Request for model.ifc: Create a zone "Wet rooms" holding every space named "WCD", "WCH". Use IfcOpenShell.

First a look at what the model holds.

```python
import ifcopenshell

model = ifcopenshell.open("model.ifc")
print(model.schema)
seen = {}
for space in model.by_type("IfcSpace"):
    seen[space.LongName] = seen.get(space.LongName, 0) + 1
for name, count in sorted(seen.items(), key=str):
    print(count, "x", name)
print("zones:", [z.Name for z in model.by_type("IfcZone")][:20])
```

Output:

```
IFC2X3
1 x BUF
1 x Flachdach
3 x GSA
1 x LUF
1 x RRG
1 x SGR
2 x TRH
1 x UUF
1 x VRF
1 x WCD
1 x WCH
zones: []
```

```python
import ifcopenshell
import ifcopenshell.api.group
import ifcopenshell.api.root

model = ifcopenshell.open("model.ifc")

names = {"WCD", "WCH"}
spaces = [s for s in model.by_type("IfcSpace") if s.LongName in names]

zone = ifcopenshell.api.root.create_entity(model, ifc_class="IfcZone", name="Wet rooms")
ifcopenshell.api.group.assign_group(model, products=spaces, group=zone)
print(len(spaces), "spaces in", zone.Name)

model.write("model_v2.ifc")
```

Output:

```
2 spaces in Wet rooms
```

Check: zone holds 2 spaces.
